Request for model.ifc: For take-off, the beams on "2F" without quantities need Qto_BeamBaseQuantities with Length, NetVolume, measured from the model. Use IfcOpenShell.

First a look at what the model holds.

```python
import ifcopenshell
import ifcopenshell.util.element
import ifcopenshell.util.unit

model = ifcopenshell.open("model.ifc")
print(model.schema)
for unit_type in ("LENGTHUNIT", "AREAUNIT", "VOLUMEUNIT"):
    print(unit_type, ifcopenshell.util.unit.calculate_unit_scale(model, unit_type))
storey = next(s for s in model.by_type("IfcBuildingStorey") if s.Name == "2F")
beams = [e for e in ifcopenshell.util.element.get_decomposition(storey) if e.is_a("IfcBeam")]
for e in sorted(beams, key=lambda e: e.id()):
    print(e.id(), e.is_a(), e.Name, list(ifcopenshell.util.element.get_psets(e, qtos_only=True)), sep=" | ")
```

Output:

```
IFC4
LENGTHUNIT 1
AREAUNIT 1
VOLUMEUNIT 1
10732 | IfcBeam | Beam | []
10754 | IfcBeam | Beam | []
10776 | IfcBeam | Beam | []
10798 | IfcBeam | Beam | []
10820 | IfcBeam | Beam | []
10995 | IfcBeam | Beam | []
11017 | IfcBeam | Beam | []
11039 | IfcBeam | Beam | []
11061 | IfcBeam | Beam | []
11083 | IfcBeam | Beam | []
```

```python
import ifcopenshell
import ifcopenshell.api.pset
import ifcopenshell.geom
import ifcopenshell.util.element
import ifcopenshell.util.shape
import ifcopenshell.util.unit

model = ifcopenshell.open("model.ifc")
unit_scale = ifcopenshell.util.unit.calculate_unit_scale(model)
volume_scale = ifcopenshell.util.unit.calculate_unit_scale(model, "VOLUMEUNIT")
settings = ifcopenshell.geom.settings()

storey = next(s for s in model.by_type("IfcBuildingStorey") if s.Name == "2F")
beams = [e for e in ifcopenshell.util.element.get_decomposition(storey) if e.is_a("IfcBeam")]

for e in sorted(beams, key=lambda e: e.id()):
    if ifcopenshell.util.element.get_psets(e, qtos_only=True, should_inherit=False):
        continue
    # Geometry comes back in metres, in the element's own axes.
    shape = ifcopenshell.geom.create_shape(settings, e)
    values = {
        "Length": ifcopenshell.util.shape.get_max_xyz(shape.geometry) / unit_scale,
        "NetVolume": ifcopenshell.util.shape.get_volume(shape.geometry) / volume_scale,
    }
    qto = ifcopenshell.api.pset.add_qto(model, product=e, name="Qto_BeamBaseQuantities")
    ifcopenshell.api.pset.edit_qto(model, qto=qto, properties=values)
    print(e.id(), {k: round(v, 3) for k, v in values.items()})

model.write("model_edited.ifc")
```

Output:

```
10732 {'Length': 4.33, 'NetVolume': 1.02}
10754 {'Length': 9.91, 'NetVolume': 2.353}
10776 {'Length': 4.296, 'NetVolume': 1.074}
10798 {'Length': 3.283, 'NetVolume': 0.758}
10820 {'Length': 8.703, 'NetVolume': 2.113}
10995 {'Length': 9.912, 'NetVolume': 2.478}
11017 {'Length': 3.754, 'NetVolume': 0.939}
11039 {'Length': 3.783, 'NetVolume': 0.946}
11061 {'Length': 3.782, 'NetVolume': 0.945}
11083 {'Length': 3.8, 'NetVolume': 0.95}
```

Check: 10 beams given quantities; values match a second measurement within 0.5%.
